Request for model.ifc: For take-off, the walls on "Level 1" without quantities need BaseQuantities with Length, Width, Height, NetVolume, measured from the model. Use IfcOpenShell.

First a look at what the model holds.

```python
import ifcopenshell
import ifcopenshell.util.element
import ifcopenshell.util.unit

model = ifcopenshell.open("model.ifc")
print(model.schema)
for unit_type in ("LENGTHUNIT", "AREAUNIT", "VOLUMEUNIT"):
    print(unit_type, ifcopenshell.util.unit.calculate_unit_scale(model, unit_type))
storey = next(s for s in model.by_type("IfcBuildingStorey") if s.Name == "Level 1")
walls = [e for e in ifcopenshell.util.element.get_decomposition(storey) if e.is_a("IfcWall")]
for e in sorted(walls, key=lambda e: e.id()):
    print(e.id(), e.is_a(), e.Name, list(ifcopenshell.util.element.get_psets(e, qtos_only=True)), sep=" | ")
```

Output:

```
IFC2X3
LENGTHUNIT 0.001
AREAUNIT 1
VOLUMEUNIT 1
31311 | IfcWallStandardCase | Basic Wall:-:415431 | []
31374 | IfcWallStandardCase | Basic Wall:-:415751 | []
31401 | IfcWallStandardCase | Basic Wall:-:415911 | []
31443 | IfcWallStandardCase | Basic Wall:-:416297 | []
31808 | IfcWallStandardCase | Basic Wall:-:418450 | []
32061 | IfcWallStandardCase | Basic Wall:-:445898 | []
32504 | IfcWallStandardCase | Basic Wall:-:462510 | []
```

```python
import ifcopenshell
import ifcopenshell.api.pset
import ifcopenshell.geom
import ifcopenshell.util.element
import ifcopenshell.util.shape
import ifcopenshell.util.unit

model = ifcopenshell.open("model.ifc")
unit_scale = ifcopenshell.util.unit.calculate_unit_scale(model)
volume_scale = ifcopenshell.util.unit.calculate_unit_scale(model, "VOLUMEUNIT")
settings = ifcopenshell.geom.settings()

storey = next(s for s in model.by_type("IfcBuildingStorey") if s.Name == "Level 1")
walls = [e for e in ifcopenshell.util.element.get_decomposition(storey) if e.is_a("IfcWall")]

for e in sorted(walls, key=lambda e: e.id()):
    if ifcopenshell.util.element.get_psets(e, qtos_only=True, should_inherit=False):
        continue
    # Geometry comes back in metres, in the element's own axes.
    shape = ifcopenshell.geom.create_shape(settings, e)
    values = {
        "Length": ifcopenshell.util.shape.get_x(shape.geometry) / unit_scale,
        "Width": ifcopenshell.util.shape.get_y(shape.geometry) / unit_scale,
        "Height": ifcopenshell.util.shape.get_z(shape.geometry) / unit_scale,
        "NetVolume": ifcopenshell.util.shape.get_volume(shape.geometry) / volume_scale,
    }
    qto = ifcopenshell.api.pset.add_qto(model, product=e, name="BaseQuantities")
    ifcopenshell.api.pset.edit_qto(model, qto=qto, properties=values)
    print(e.id(), {k: round(v, 3) for k, v in values.items()})

model.write("model_v2.ifc")
```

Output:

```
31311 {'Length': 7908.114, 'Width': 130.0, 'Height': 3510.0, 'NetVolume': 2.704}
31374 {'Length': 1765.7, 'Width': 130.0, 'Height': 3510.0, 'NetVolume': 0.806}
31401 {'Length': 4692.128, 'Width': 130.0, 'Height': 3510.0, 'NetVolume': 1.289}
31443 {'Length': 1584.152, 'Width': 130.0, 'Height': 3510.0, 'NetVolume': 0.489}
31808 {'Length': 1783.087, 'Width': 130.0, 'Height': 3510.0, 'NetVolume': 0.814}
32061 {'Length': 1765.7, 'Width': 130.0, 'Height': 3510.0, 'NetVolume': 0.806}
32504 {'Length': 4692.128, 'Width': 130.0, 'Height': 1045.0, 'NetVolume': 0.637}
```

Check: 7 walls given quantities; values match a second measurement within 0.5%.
